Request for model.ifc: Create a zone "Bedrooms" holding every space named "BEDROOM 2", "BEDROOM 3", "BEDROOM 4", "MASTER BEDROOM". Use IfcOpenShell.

First a look at what the model holds.

```python
import ifcopenshell

model = ifcopenshell.open("model.ifc")
print(model.schema)
seen = {}
for space in model.by_type("IfcSpace"):
    seen[space.LongName] = seen.get(space.LongName, 0) + 1
for name, count in sorted(seen.items(), key=str):
    print(count, "x", name)
print("zones:", [z.Name for z in model.by_type("IfcZone")][:20])
```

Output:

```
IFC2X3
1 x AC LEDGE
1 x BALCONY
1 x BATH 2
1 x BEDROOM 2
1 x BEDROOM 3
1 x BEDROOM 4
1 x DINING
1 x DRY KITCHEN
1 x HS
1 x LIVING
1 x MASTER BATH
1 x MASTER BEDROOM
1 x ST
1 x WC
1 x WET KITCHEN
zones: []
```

```python
import ifcopenshell
import ifcopenshell.api.group
import ifcopenshell.api.root

model = ifcopenshell.open("model.ifc")

names = {"BEDROOM 2", "BEDROOM 3", "BEDROOM 4", "MASTER BEDROOM"}
spaces = [s for s in model.by_type("IfcSpace") if s.LongName in names]

zone = ifcopenshell.api.root.create_entity(model, ifc_class="IfcZone", name="Bedrooms")
ifcopenshell.api.group.assign_group(model, products=spaces, group=zone)
print(len(spaces), "spaces in", zone.Name)

model.write("model_updated.ifc")
```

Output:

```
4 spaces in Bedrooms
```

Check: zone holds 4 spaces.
